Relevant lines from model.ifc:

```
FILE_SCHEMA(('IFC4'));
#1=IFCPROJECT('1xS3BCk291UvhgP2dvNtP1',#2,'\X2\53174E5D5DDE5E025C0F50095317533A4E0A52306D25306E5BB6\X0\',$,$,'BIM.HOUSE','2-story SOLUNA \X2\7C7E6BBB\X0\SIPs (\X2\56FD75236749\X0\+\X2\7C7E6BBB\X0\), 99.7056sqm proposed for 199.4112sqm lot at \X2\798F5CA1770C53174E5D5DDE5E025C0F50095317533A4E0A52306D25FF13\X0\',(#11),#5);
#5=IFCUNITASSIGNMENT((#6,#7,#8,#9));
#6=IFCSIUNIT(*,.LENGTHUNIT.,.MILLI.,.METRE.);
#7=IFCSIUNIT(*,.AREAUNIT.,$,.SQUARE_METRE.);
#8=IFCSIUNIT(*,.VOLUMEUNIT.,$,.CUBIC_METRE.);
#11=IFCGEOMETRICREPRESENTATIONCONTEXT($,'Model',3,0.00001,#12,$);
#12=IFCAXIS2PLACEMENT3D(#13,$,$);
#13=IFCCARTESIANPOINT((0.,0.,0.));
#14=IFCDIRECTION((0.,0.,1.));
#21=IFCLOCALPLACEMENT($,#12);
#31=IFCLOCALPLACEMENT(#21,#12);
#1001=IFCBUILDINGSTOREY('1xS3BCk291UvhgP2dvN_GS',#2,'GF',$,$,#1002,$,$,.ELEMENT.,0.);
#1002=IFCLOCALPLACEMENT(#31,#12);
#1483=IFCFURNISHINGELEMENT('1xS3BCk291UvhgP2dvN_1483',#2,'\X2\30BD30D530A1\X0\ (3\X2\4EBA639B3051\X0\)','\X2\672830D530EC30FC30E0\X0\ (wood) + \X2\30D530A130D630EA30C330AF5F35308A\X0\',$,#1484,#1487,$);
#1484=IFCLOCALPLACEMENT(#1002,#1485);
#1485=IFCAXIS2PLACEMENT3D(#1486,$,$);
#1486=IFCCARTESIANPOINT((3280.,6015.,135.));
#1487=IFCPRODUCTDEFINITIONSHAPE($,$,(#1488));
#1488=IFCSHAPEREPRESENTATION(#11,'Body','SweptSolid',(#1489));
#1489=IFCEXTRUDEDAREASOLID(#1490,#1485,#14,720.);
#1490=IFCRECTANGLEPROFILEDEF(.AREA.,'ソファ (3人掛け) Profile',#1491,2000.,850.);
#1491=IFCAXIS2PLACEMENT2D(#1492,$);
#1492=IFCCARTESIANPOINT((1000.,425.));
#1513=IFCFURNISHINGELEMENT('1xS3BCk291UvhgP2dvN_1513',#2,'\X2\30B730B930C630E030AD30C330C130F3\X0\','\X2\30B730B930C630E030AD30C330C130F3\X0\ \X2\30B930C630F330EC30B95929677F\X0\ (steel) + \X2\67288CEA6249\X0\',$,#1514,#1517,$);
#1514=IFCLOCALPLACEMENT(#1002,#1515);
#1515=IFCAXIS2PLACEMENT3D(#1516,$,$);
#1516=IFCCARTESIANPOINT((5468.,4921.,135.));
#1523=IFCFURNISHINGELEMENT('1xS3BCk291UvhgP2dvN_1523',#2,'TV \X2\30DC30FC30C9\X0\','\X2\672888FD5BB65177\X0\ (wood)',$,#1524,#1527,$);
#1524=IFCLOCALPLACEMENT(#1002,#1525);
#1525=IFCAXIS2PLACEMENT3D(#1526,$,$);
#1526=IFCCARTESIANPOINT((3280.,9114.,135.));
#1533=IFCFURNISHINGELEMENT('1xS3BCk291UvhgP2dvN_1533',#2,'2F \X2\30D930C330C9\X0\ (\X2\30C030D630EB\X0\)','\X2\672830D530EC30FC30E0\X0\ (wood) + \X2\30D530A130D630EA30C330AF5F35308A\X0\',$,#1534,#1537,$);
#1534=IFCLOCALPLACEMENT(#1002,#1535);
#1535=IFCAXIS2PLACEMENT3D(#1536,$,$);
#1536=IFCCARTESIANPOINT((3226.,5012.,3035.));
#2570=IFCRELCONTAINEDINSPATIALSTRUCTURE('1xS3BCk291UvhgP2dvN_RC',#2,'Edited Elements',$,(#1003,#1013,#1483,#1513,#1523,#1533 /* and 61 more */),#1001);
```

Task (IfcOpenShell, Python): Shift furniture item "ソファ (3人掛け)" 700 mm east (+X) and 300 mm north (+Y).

```python
import ifcopenshell
import ifcopenshell.api.geometry
import ifcopenshell.util.placement

model = ifcopenshell.open("model.ifc")

item = model.by_guid("1xS3BCk291UvhgP2dvN_1483")
matrix = ifcopenshell.util.placement.get_local_placement(item.ObjectPlacement)
matrix[0, 3] += 700.0
matrix[1, 3] += 300.0
ifcopenshell.api.geometry.edit_object_placement(model, product=item, matrix=matrix, is_si=False)

print(ifcopenshell.util.placement.get_local_placement(item.ObjectPlacement).round(3) + 0.0)

model.write("model_rev.ifc")
```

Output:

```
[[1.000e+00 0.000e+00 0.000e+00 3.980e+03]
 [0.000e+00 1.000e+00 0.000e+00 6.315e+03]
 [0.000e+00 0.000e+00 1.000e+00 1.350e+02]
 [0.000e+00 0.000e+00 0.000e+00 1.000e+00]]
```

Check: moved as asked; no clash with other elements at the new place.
